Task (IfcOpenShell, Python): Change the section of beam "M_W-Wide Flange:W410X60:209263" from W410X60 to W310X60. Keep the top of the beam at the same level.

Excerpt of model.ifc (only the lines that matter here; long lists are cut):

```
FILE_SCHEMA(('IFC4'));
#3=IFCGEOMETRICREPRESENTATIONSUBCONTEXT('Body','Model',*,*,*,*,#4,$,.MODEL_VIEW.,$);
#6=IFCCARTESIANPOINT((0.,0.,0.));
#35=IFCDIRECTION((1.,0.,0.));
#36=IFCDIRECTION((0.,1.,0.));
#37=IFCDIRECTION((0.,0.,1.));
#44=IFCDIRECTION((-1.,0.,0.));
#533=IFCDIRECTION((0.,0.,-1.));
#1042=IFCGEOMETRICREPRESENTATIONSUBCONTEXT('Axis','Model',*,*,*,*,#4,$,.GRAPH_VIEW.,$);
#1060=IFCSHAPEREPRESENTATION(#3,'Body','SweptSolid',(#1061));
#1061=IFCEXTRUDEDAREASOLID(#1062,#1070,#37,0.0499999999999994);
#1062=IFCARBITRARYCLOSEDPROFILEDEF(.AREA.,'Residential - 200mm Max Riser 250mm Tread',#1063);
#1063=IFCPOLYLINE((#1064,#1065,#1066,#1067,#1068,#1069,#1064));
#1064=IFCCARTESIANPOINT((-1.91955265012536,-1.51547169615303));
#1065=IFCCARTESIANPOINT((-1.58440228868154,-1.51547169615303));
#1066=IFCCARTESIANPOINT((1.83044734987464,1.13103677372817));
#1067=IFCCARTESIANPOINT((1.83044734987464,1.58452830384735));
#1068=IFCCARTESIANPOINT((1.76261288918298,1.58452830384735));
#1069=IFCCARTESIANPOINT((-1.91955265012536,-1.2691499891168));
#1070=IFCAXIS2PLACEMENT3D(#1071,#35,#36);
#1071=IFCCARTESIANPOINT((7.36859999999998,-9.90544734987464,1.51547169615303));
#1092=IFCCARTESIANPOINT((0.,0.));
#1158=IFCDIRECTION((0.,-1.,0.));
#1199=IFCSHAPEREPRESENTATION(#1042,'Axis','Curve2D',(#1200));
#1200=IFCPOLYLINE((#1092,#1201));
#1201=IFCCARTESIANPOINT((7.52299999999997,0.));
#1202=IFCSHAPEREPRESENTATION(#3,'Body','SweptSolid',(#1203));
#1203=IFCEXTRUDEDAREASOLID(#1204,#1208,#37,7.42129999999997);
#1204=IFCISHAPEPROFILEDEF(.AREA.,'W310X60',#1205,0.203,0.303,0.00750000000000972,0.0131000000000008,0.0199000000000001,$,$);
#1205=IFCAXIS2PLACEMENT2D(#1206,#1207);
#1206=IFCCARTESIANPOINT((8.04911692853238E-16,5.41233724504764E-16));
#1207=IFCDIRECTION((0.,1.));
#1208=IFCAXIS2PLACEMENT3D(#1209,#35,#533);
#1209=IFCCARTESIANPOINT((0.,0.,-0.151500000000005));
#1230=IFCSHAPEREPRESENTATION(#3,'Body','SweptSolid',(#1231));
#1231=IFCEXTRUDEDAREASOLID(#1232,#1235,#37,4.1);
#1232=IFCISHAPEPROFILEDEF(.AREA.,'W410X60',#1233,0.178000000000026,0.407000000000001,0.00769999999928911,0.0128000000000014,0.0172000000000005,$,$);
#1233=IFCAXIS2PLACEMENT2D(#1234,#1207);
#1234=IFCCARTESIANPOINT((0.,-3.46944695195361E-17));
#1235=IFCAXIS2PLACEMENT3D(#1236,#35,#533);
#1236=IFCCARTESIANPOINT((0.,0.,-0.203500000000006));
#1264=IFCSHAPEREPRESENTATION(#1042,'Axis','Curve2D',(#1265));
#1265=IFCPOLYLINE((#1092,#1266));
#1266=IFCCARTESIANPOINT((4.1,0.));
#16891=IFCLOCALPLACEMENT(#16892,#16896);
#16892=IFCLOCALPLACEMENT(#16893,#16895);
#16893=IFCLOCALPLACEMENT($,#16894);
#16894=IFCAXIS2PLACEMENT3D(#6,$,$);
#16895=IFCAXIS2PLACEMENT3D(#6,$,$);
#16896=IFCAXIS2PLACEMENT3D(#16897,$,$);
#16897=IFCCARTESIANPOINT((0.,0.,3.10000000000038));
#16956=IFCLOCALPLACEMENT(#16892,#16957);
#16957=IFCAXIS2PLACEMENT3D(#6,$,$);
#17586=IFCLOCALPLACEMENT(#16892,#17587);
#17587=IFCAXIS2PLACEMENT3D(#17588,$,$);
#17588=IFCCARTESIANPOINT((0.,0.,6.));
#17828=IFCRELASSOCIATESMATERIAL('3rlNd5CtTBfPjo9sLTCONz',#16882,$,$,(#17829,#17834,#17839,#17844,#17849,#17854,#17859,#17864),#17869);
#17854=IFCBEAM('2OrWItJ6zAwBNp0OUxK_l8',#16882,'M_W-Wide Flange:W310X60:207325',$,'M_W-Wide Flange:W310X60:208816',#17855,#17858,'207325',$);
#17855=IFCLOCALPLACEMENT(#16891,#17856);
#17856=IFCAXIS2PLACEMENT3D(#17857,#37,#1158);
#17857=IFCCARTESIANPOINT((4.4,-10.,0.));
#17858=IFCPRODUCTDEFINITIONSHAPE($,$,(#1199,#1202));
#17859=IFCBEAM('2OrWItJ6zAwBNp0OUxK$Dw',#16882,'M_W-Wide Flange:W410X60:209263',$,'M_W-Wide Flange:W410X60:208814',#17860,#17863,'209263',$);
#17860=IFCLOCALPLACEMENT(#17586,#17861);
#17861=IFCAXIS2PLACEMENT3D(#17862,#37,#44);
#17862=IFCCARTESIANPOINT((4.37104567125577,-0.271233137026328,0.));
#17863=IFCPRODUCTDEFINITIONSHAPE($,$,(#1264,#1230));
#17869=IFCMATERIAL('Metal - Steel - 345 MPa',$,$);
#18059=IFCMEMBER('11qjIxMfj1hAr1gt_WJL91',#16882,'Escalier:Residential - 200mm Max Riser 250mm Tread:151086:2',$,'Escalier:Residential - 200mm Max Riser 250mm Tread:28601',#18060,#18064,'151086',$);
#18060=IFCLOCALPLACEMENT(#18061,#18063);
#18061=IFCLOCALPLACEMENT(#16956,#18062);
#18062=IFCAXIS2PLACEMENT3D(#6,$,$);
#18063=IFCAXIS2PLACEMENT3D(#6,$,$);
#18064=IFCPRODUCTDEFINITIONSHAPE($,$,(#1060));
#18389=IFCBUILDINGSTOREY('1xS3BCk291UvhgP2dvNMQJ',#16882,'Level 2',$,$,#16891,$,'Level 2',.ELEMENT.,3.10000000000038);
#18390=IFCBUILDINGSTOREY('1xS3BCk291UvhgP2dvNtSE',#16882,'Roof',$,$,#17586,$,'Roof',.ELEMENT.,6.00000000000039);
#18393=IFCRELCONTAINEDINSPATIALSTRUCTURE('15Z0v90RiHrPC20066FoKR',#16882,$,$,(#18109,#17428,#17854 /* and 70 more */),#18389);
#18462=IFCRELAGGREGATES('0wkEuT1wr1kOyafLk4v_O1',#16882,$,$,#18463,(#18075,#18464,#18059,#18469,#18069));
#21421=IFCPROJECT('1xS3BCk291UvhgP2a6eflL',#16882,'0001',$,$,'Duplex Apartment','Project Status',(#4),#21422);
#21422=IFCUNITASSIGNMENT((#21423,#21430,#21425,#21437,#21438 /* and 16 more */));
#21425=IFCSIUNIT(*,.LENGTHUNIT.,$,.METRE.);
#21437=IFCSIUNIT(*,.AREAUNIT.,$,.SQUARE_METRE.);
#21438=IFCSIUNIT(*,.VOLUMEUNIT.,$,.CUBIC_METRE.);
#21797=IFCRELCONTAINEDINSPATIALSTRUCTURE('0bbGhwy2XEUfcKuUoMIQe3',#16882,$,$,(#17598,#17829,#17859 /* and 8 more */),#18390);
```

```python
import ifcopenshell
import ifcopenshell.util.element
import ifcopenshell.util.representation

model = ifcopenshell.open("model.ifc")

member = model.by_id(17859)
source = next(p for p in model.by_type("IfcIShapeProfileDef") if p.ProfileName == "W310X60")

body = ifcopenshell.util.representation.get_representation(member, "Model", "Body")
solid = body.Items[0]
old_profile = solid.SweptArea

# Copy the section's sizes but keep this member's own profile position.
profile = ifcopenshell.util.element.copy(model, source)
# Profiles are centred, so shift by half the change in depth to hold the top.
shift = (old_profile.OverallDepth - profile.OverallDepth) / 2
x, y = old_profile.Position.Location.Coordinates
up = (-1.0, 0.0)  # upwards, in the solid's own plane
location = model.createIfcCartesianPoint((x + up[0] * shift, y + up[1] * shift))
profile.Position = model.createIfcAxis2Placement2D(location, old_profile.Position.RefDirection)
solid.SweptArea = profile
if not model.get_total_inverses(old_profile):
    ifcopenshell.util.element.remove_deep2(model, old_profile)
member.Name = member.Name.replace("W410X60", "W310X60")
member.ObjectType = member.ObjectType.replace("W410X60", "W310X60")

print(solid.SweptArea)

model.write("model_edited.ifc")
```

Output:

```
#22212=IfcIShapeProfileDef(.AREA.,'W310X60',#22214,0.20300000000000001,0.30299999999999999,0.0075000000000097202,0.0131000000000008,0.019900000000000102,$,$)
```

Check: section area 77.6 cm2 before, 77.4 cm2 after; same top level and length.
